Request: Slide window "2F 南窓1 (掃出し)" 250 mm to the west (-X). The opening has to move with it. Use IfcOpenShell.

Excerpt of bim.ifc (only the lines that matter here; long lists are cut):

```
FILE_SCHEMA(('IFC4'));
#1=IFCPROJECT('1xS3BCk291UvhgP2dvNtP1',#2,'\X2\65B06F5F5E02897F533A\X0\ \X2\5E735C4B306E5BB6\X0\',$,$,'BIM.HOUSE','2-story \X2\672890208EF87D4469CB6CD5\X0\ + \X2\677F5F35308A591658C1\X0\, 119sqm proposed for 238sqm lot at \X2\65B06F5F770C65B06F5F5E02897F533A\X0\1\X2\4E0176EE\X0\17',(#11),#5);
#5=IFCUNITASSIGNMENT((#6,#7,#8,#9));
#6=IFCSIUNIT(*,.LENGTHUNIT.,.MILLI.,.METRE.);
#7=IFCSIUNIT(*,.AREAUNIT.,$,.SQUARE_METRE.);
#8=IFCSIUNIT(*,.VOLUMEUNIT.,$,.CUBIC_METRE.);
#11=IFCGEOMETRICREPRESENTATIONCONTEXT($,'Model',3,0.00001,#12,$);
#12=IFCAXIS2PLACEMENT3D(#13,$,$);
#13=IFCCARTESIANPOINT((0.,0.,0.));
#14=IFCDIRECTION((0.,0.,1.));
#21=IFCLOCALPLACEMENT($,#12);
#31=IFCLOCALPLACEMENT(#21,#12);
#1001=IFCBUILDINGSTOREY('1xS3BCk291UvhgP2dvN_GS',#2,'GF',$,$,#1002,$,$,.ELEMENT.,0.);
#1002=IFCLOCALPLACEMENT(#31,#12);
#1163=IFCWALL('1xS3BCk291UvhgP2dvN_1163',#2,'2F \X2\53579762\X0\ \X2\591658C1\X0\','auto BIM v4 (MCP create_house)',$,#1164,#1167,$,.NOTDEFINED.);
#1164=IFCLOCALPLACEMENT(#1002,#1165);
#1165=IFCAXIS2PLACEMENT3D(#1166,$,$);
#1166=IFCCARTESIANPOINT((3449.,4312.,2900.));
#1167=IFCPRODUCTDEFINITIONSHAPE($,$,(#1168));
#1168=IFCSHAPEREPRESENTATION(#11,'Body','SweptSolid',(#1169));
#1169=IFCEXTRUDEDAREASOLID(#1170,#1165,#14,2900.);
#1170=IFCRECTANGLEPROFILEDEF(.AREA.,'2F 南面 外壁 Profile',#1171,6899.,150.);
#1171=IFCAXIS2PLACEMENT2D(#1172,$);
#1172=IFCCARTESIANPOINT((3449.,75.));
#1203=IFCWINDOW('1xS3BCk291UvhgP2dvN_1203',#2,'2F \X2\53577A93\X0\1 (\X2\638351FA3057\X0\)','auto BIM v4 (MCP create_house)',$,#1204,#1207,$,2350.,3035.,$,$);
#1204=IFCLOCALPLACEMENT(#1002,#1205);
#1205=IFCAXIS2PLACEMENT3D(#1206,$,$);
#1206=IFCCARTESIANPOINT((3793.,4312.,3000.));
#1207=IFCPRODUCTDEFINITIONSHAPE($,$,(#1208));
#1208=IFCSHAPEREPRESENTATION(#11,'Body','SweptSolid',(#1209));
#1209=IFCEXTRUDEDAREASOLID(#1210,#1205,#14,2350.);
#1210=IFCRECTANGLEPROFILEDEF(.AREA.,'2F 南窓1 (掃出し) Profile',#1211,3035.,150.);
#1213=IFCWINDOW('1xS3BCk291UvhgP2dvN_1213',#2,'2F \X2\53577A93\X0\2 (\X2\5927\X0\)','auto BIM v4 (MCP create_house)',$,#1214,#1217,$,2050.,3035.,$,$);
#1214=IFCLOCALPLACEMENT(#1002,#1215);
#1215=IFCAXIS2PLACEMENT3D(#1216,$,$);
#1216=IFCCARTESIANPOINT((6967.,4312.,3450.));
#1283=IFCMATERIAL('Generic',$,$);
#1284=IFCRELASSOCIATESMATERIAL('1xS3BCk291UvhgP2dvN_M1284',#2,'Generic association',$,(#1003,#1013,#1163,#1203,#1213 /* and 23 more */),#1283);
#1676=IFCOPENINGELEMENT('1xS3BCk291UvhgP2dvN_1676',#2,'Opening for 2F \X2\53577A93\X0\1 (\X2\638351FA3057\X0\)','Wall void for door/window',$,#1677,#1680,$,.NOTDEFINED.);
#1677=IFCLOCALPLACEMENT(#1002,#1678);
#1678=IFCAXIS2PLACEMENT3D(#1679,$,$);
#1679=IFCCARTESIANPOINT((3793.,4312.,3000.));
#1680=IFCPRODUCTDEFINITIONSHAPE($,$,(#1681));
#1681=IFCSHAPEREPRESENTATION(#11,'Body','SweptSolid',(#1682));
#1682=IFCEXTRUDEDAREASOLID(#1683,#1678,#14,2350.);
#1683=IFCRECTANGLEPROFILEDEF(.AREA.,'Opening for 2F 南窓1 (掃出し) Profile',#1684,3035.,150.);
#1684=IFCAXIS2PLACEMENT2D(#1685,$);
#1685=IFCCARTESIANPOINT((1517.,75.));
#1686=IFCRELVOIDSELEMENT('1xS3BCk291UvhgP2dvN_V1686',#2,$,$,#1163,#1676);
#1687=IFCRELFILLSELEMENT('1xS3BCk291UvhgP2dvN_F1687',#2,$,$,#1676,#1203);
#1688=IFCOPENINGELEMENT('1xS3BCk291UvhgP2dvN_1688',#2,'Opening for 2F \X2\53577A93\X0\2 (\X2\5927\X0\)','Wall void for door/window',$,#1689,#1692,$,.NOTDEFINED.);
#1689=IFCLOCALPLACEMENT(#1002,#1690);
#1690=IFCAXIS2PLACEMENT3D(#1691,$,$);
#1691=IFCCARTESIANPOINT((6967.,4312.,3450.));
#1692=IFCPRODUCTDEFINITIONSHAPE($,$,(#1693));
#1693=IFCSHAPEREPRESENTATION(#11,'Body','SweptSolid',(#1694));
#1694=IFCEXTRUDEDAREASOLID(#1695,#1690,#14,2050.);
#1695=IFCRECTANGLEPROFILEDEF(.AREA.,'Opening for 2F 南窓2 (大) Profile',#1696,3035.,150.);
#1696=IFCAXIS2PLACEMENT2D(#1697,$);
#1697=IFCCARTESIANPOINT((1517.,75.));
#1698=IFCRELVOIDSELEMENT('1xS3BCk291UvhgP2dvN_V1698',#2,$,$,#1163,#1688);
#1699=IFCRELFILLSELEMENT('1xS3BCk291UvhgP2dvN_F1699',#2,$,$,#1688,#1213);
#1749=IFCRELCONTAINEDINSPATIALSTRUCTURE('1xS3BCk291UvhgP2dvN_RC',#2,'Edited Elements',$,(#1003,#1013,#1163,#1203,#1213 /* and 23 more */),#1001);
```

```python
import ifcopenshell
import ifcopenshell.api.geometry
import ifcopenshell.util.placement
import ifcopenshell.util.unit

model = ifcopenshell.open("bim.ifc")
unit_scale = ifcopenshell.util.unit.calculate_unit_scale(model)

window = model.by_id(1203)
opening = window.FillsVoids[0].RelatingOpeningElement
wall = opening.VoidsElements[0].RelatingBuildingElement

wall_matrix = ifcopenshell.util.placement.get_local_placement(wall.ObjectPlacement)
shift = wall_matrix[:3, 0] * -0.25 / unit_scale
before = ifcopenshell.util.placement.get_local_placement(window.ObjectPlacement)[:3, 3].copy()

# The window is not placed relative to its opening, so move both.
for product in (opening, window):
    matrix = ifcopenshell.util.placement.get_local_placement(product.ObjectPlacement)
    matrix[:3, 3] += shift
    ifcopenshell.api.geometry.edit_object_placement(model, product=product, matrix=matrix, is_si=False)

after = ifcopenshell.util.placement.get_local_placement(window.ObjectPlacement)[:3, 3]
print("window moved by", (after - before).round(3) + 0.0)

model.write("bim_edited.ifc")
```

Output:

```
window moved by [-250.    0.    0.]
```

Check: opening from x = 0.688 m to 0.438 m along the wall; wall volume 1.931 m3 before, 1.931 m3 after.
